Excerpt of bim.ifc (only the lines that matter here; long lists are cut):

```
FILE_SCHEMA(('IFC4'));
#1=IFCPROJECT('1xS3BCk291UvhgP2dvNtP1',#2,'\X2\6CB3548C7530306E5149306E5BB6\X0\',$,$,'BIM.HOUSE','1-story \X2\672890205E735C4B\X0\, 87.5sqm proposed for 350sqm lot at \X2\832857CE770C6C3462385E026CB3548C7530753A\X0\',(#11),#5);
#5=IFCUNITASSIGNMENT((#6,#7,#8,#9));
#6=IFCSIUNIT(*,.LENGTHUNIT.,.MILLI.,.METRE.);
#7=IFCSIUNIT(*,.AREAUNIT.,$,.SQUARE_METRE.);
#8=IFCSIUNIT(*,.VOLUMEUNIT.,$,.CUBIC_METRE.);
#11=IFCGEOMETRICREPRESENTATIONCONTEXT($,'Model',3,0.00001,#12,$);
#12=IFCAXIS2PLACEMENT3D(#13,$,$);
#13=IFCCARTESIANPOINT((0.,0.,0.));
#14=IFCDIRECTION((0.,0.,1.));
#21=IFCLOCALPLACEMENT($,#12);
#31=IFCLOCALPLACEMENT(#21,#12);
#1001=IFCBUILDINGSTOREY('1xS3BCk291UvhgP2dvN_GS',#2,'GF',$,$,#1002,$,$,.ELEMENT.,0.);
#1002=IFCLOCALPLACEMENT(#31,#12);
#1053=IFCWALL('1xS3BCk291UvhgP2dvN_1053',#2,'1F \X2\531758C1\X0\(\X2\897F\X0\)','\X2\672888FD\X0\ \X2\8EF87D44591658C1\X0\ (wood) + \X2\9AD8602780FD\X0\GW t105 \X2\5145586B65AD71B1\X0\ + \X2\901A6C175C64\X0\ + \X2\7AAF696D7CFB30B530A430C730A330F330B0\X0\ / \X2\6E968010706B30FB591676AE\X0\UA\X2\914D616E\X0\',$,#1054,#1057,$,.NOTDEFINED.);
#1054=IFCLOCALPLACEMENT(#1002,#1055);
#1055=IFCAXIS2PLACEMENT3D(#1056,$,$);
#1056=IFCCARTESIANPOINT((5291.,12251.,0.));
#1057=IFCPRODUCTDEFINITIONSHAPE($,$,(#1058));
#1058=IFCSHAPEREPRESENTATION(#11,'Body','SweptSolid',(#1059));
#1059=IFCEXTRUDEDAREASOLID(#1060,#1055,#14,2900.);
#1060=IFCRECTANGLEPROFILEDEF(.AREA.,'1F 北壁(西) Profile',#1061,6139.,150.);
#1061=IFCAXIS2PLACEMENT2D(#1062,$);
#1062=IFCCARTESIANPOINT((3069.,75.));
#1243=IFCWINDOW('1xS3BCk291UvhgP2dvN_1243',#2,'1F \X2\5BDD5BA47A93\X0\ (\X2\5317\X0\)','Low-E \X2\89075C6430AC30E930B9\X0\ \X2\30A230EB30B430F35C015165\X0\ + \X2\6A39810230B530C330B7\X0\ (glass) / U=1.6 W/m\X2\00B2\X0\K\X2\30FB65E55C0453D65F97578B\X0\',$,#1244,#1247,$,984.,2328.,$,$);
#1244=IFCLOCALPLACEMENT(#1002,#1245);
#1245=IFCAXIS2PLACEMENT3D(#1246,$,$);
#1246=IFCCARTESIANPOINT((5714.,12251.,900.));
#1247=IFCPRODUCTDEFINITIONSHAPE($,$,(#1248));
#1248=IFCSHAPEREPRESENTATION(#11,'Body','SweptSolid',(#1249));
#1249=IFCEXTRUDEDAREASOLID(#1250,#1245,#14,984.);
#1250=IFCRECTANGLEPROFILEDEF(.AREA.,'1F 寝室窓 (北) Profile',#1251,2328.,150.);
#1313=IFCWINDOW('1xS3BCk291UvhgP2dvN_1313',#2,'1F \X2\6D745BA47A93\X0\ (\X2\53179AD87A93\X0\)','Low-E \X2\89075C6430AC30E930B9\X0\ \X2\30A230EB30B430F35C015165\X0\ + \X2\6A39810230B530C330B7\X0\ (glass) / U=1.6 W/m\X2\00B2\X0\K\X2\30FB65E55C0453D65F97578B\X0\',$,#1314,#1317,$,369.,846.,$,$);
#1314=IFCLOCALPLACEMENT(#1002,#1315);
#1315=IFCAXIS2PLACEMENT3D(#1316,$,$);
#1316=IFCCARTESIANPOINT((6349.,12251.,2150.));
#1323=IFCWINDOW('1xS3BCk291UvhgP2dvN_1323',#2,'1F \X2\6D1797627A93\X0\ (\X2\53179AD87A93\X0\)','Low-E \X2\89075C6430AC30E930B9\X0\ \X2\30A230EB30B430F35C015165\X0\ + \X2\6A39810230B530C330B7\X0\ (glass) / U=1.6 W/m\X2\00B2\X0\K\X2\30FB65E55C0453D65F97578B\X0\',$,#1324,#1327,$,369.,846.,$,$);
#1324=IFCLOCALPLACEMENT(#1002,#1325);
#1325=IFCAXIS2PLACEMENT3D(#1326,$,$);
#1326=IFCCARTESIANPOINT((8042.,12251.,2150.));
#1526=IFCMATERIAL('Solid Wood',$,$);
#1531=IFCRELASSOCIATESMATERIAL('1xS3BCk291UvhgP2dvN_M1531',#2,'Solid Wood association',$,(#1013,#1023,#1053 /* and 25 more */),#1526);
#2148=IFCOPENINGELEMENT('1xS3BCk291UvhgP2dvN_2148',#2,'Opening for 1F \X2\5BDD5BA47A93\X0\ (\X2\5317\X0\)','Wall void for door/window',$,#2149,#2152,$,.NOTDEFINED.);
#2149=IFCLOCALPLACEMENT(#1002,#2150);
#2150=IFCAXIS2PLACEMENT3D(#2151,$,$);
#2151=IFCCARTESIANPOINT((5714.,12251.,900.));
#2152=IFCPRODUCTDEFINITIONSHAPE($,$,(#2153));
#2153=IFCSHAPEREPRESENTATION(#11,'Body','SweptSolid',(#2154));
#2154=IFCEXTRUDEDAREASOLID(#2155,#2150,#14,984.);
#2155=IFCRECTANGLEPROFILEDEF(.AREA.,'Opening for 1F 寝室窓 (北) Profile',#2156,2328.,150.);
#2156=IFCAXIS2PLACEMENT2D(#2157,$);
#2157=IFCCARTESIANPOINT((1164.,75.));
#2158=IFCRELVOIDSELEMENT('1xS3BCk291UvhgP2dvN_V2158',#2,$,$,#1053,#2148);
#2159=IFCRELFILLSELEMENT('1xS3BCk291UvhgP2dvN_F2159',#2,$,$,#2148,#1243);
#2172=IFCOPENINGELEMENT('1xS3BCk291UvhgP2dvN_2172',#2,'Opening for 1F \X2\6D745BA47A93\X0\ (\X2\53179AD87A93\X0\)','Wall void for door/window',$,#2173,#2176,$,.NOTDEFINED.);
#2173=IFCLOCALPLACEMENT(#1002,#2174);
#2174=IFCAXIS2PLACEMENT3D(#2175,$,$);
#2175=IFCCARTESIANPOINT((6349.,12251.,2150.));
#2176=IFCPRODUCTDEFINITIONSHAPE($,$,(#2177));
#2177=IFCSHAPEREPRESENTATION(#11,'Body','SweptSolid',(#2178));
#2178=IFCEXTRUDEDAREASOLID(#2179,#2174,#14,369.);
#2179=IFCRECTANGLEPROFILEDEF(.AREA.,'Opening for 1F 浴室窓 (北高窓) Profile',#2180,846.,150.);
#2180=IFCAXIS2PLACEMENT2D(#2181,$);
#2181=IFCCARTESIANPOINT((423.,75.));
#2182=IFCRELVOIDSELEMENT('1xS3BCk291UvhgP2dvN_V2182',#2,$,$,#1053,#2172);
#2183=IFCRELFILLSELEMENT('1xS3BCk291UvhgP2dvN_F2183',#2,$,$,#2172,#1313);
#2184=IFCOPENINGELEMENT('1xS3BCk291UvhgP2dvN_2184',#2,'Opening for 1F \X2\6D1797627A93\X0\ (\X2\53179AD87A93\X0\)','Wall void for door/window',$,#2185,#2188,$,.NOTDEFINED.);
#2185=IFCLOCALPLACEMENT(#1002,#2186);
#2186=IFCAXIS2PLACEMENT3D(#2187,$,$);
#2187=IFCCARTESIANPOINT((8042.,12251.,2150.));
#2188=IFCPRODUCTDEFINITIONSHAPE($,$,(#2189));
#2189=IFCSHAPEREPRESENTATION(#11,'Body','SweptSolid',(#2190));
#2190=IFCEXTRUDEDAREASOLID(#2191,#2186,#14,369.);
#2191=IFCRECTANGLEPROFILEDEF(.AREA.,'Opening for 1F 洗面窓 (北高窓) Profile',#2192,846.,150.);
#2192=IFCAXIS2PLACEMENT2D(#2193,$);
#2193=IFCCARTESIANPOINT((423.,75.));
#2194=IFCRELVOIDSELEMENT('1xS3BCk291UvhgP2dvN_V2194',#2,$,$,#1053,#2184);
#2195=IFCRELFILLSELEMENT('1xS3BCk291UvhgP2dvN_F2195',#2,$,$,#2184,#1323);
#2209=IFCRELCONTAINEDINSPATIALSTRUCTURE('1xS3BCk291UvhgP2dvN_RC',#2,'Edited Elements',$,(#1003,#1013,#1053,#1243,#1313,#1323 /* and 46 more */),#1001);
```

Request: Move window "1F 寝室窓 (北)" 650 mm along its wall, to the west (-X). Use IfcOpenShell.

```python
import ifcopenshell
import ifcopenshell.api.geometry
import ifcopenshell.util.placement

model = ifcopenshell.open("bim.ifc")

window = model.by_guid("1xS3BCk291UvhgP2dvN_1243")
opening = window.FillsVoids[0].RelatingOpeningElement
wall = opening.VoidsElements[0].RelatingBuildingElement

wall_matrix = ifcopenshell.util.placement.get_local_placement(wall.ObjectPlacement)
shift = wall_matrix[:3, 0] * -650.0
before = ifcopenshell.util.placement.get_local_placement(window.ObjectPlacement)[:3, 3].copy()

# The window is not placed relative to its opening, so move both.
for product in (opening, window):
    matrix = ifcopenshell.util.placement.get_local_placement(product.ObjectPlacement)
    matrix[:3, 3] += shift
    ifcopenshell.api.geometry.edit_object_placement(model, product=product, matrix=matrix, is_si=False)

after = ifcopenshell.util.placement.get_local_placement(window.ObjectPlacement)[:3, 3]
print("window moved by", (after - before).round(3) + 0.0)

model.write("bim_v2.ifc")
```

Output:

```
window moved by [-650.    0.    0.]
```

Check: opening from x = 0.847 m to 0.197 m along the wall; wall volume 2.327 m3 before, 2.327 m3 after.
